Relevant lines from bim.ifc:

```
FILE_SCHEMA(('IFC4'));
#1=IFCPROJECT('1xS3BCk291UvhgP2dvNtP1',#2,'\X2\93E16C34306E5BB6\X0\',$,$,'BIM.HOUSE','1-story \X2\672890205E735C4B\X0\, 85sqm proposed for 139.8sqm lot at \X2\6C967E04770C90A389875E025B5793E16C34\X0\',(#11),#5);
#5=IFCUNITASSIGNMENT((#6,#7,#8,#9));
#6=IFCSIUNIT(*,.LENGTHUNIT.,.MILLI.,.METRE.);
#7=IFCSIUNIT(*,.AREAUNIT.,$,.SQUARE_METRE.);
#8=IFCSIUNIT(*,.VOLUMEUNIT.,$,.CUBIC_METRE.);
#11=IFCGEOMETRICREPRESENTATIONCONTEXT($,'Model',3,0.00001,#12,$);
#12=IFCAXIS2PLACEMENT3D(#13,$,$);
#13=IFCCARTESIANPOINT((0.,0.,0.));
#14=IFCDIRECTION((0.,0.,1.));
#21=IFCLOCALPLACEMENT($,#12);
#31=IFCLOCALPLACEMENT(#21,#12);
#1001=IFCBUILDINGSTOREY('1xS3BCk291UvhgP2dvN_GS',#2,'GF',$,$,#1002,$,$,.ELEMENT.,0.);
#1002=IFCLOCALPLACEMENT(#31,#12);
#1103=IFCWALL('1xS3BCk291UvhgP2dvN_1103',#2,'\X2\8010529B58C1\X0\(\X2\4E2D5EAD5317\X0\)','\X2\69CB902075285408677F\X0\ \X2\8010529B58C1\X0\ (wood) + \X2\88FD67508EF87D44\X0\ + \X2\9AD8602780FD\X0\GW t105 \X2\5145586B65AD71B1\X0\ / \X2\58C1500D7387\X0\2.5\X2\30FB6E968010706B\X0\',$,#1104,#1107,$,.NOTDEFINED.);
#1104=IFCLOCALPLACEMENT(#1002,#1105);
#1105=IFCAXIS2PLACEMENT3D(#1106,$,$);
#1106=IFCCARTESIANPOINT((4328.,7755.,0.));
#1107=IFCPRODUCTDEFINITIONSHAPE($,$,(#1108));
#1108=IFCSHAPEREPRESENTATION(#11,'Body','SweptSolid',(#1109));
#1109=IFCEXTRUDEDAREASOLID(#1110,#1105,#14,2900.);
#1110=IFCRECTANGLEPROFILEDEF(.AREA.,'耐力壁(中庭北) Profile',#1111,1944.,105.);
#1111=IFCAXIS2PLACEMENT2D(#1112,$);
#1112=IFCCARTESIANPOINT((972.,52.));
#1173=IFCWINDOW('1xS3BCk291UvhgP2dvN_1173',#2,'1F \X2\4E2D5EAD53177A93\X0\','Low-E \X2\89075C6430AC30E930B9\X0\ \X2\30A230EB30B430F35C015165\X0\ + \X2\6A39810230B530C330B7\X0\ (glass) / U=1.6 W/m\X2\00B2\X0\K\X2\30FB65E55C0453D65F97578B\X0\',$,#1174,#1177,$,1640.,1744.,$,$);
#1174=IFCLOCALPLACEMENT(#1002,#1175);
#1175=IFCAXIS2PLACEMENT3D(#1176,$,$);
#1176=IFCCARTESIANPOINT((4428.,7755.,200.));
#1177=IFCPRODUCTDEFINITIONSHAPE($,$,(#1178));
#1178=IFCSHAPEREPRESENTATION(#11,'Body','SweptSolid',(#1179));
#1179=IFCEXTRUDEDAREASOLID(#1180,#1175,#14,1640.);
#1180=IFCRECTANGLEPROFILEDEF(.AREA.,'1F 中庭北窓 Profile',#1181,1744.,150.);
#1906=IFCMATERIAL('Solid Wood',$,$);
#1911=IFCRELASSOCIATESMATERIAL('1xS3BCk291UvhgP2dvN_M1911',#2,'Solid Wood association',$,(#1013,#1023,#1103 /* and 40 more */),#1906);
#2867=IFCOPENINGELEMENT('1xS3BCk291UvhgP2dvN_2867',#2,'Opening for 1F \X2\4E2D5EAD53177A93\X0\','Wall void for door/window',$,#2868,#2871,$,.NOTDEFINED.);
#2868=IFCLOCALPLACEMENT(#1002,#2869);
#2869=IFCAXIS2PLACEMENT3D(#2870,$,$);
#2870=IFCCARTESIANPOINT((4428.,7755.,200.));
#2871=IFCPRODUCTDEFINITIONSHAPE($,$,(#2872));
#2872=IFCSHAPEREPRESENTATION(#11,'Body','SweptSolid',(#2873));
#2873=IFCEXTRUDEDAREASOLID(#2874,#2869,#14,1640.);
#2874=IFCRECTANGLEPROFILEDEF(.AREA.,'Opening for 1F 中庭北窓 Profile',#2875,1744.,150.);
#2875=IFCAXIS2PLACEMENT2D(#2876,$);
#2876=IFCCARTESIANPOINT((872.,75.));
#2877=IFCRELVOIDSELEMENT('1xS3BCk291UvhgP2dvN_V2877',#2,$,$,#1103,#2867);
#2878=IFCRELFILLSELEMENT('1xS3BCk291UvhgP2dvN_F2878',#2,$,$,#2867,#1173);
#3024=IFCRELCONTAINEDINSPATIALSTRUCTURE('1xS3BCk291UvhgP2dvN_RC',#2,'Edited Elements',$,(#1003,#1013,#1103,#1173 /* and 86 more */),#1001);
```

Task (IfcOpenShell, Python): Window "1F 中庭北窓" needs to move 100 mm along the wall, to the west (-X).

```python
import ifcopenshell
import ifcopenshell.api.geometry
import ifcopenshell.util.placement
import ifcopenshell.util.unit

model = ifcopenshell.open("bim.ifc")
unit_scale = ifcopenshell.util.unit.calculate_unit_scale(model)

window = model.by_guid("1xS3BCk291UvhgP2dvN_1173")
opening = window.FillsVoids[0].RelatingOpeningElement
wall = opening.VoidsElements[0].RelatingBuildingElement

wall_matrix = ifcopenshell.util.placement.get_local_placement(wall.ObjectPlacement)
shift = wall_matrix[:3, 0] * -0.1 / unit_scale
before = ifcopenshell.util.placement.get_local_placement(window.ObjectPlacement)[:3, 3].copy()

# The window is not placed relative to its opening, so move both.
for product in (opening, window):
    matrix = ifcopenshell.util.placement.get_local_placement(product.ObjectPlacement)
    matrix[:3, 3] += shift
    ifcopenshell.api.geometry.edit_object_placement(model, product=product, matrix=matrix, is_si=False)

after = ifcopenshell.util.placement.get_local_placement(window.ObjectPlacement)[:3, 3]
print("window moved by", (after - before).round(3) + 0.0)

model.write("bim_v2.ifc")
```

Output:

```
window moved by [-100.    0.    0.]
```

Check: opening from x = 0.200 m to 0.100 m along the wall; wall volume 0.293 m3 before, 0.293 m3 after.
